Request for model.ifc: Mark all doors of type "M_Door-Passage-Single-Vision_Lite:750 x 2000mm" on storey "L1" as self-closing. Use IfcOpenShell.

First a look at what the model holds.

```python
import ifcopenshell
import ifcopenshell.util.element

model = ifcopenshell.open("model.ifc")
print(model.schema)
storey = next(s for s in model.by_type("IfcBuildingStorey") if s.Name == "L1")
doors = [e for e in ifcopenshell.util.element.get_decomposition(storey) if e.is_a("IfcDoor")]
seen = {}
for e in doors:
    element_type = ifcopenshell.util.element.get_type(e)
    key = (element_type.Name if element_type != e and element_type else None, ifcopenshell.util.element.get_pset(e, "Pset_DoorCommon", "SelfClosing"))
    seen[key] = seen.get(key, 0) + 1
for (name, value), count in sorted(seen.items(), key=str):
    print(count, "x", name, "|", value)
```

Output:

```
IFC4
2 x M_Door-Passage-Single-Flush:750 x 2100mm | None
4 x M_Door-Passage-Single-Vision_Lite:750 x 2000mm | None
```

```python
import ifcopenshell
import ifcopenshell.api.pset
import ifcopenshell.util.element

model = ifcopenshell.open("model.ifc")

storey = next(s for s in model.by_type("IfcBuildingStorey") if s.Name == "L1")
doors = [e for e in ifcopenshell.util.element.get_decomposition(storey) if e.is_a("IfcDoor")]

count = 0
for e in doors:
    element_type = ifcopenshell.util.element.get_type(e)
    if element_type in (None, e) or element_type.Name != "M_Door-Passage-Single-Vision_Lite:750 x 2000mm":
        continue
    # add_pset returns the element's existing set when there is one.
    pset = ifcopenshell.api.pset.add_pset(model, product=e, name="Pset_DoorCommon")
    ifcopenshell.api.pset.edit_pset(model, pset=pset, properties={"SelfClosing": True})
    count += 1

print(count, "doors updated")

model.write("model-out.ifc")
```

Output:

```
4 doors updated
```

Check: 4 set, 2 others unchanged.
